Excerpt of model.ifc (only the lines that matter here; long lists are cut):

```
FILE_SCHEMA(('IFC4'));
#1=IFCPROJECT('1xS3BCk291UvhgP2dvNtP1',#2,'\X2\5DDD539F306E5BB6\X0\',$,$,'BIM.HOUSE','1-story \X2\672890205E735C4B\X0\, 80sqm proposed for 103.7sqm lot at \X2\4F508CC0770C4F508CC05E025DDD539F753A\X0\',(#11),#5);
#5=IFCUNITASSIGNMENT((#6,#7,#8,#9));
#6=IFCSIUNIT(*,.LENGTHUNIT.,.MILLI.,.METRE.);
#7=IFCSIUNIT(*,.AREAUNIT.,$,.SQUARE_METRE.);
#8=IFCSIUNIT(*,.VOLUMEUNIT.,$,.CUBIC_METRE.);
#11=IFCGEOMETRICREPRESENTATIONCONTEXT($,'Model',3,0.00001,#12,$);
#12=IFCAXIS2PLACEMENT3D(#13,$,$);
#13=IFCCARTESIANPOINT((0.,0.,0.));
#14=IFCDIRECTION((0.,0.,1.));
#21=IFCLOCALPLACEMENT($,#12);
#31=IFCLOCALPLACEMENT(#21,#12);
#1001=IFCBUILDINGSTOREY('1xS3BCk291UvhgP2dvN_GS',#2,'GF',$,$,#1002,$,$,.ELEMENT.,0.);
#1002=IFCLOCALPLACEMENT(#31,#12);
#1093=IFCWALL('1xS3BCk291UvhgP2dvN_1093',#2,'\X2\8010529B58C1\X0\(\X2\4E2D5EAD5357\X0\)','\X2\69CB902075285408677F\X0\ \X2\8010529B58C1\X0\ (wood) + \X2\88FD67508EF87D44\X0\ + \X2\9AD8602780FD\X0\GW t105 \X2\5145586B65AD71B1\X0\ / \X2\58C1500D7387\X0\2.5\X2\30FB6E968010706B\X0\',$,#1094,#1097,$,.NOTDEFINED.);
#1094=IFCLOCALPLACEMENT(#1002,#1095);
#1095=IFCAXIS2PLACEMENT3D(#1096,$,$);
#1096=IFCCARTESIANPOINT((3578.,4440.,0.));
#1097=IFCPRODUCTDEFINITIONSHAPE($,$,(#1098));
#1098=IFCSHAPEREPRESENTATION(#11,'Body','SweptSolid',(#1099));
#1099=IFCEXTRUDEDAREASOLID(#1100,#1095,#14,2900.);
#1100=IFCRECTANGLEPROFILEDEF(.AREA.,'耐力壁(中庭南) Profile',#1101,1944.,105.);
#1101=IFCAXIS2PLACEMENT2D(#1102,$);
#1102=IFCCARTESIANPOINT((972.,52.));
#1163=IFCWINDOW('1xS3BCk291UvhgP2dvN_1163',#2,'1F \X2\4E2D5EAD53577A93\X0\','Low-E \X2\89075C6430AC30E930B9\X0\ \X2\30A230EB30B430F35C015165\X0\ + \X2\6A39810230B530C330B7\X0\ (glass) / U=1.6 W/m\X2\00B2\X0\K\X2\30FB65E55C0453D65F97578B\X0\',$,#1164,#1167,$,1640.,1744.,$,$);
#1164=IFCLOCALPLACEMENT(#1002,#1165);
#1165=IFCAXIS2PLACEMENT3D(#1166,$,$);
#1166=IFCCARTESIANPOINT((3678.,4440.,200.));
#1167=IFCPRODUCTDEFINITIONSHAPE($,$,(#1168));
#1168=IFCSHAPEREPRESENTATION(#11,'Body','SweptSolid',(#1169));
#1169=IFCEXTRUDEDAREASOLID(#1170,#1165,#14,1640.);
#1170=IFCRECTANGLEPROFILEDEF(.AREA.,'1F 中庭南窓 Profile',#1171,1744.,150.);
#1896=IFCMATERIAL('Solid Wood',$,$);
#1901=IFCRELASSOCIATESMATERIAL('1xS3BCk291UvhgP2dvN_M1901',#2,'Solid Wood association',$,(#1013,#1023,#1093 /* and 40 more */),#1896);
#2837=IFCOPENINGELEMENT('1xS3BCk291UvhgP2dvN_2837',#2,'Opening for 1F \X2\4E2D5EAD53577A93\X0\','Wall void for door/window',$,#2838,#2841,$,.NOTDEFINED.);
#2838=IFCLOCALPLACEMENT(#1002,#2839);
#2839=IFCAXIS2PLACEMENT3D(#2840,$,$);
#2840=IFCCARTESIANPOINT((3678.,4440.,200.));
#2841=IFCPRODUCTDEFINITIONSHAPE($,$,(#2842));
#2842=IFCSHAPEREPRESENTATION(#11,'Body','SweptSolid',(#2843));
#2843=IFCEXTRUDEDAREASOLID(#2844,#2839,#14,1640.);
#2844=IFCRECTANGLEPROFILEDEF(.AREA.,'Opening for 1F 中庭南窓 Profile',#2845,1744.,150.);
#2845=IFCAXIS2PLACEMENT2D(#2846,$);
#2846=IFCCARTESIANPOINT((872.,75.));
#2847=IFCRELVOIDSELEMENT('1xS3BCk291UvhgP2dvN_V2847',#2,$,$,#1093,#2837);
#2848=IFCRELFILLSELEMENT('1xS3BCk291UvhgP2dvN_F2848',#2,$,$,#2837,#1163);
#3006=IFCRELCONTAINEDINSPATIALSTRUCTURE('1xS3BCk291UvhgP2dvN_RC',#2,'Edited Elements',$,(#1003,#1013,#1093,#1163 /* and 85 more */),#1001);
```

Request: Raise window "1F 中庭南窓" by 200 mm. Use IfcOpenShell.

```python
import numpy as np
import ifcopenshell
import ifcopenshell.api.geometry
import ifcopenshell.util.placement
import ifcopenshell.util.unit

model = ifcopenshell.open("model.ifc")
unit_scale = ifcopenshell.util.unit.calculate_unit_scale(model)

window = model.by_id(1163)
opening = window.FillsVoids[0].RelatingOpeningElement
dz = 200.0

shift = np.array([0.0, 0.0, dz])
# The window is not placed relative to its opening, so move both.
for product in (opening, window):
    matrix = ifcopenshell.util.placement.get_local_placement(product.ObjectPlacement)
    matrix[:3, 3] += shift
    ifcopenshell.api.geometry.edit_object_placement(model, product=product, matrix=matrix, is_si=False)

print(f"moved by {dz * unit_scale:+.3f} m")

model.write("model_rev.ifc")
```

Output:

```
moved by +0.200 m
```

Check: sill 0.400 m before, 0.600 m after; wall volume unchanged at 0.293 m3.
